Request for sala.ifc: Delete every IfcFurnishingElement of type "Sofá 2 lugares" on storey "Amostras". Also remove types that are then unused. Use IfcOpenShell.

First a look at what the model holds.

```python
import ifcopenshell
import ifcopenshell.util.element

model = ifcopenshell.open("sala.ifc")
print(model.schema)
storey = next(s for s in model.by_type("IfcBuildingStorey") if s.Name == "Amostras")
furniture = [e for e in ifcopenshell.util.element.get_decomposition(storey) if e.is_a("IfcFurnishingElement")]
seen = {}
for e in furniture:
    element_type = ifcopenshell.util.element.get_type(e)
    name = element_type.Name if element_type not in (None, e) else None
    seen[name] = seen.get(name, 0) + 1
for name, count in sorted(seen.items(), key=str):
    print(count, "x", name)
```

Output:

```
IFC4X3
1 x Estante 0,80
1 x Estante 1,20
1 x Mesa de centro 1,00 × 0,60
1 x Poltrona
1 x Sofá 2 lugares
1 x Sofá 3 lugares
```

```python
import ifcopenshell
import ifcopenshell.api.root
import ifcopenshell.util.element

model = ifcopenshell.open("sala.ifc")

storey = next(s for s in model.by_type("IfcBuildingStorey") if s.Name == "Amostras")
furniture = [e for e in ifcopenshell.util.element.get_decomposition(storey) if e.is_a("IfcFurnishingElement")]
targets = [e for e in furniture if (t := ifcopenshell.util.element.get_type(e)) not in (None, e) and t.Name == "Sofá 2 lugares"]
types = {ifcopenshell.util.element.get_type(e) for e in targets} - {None, *targets}

for e in targets:
    ifcopenshell.api.root.remove_product(model, product=e)
print(len(targets), "removed")

unused = [t for t in types if not ifcopenshell.util.element.get_types(t)]
for t in unused:
    ifcopenshell.api.root.remove_product(model, product=t)
print(len(unused), "unused types removed")

model.write("sala_v2.ifc")
```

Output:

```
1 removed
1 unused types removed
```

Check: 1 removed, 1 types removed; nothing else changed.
